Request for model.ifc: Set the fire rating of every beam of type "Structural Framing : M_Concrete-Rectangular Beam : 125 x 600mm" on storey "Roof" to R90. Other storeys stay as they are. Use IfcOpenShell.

First a look at what the model holds.

```python
import ifcopenshell
import ifcopenshell.util.element

model = ifcopenshell.open("model.ifc")
print(model.schema)
storey = next(s for s in model.by_type("IfcBuildingStorey") if s.Name == "Roof")
beams = [e for e in ifcopenshell.util.element.get_decomposition(storey) if e.is_a("IfcBeam")]
seen = {}
for e in beams:
    element_type = ifcopenshell.util.element.get_type(e)
    key = (element_type.Name if element_type != e and element_type else None, ifcopenshell.util.element.get_pset(e, "Pset_BeamCommon", "FireRating"))
    seen[key] = seen.get(key, 0) + 1
for (name, value), count in sorted(seen.items(), key=str):
    print(count, "x", name, "|", value)
```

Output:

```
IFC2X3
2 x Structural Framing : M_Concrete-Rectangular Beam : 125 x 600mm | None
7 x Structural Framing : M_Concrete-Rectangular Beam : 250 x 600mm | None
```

```python
import ifcopenshell
import ifcopenshell.api.pset
import ifcopenshell.util.element

model = ifcopenshell.open("model.ifc")

storey = next(s for s in model.by_type("IfcBuildingStorey") if s.Name == "Roof")
beams = [e for e in ifcopenshell.util.element.get_decomposition(storey) if e.is_a("IfcBeam")]

count = 0
for e in beams:
    element_type = ifcopenshell.util.element.get_type(e)
    if element_type in (None, e) or element_type.Name != "Structural Framing : M_Concrete-Rectangular Beam : 125 x 600mm":
        continue
    # add_pset returns the element's existing set when there is one.
    pset = ifcopenshell.api.pset.add_pset(model, product=e, name="Pset_BeamCommon")
    ifcopenshell.api.pset.edit_pset(model, pset=pset, properties={"FireRating": "R90"})
    count += 1

print(count, "beams updated")

model.write("model_rev.ifc")
```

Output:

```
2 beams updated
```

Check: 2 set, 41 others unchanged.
